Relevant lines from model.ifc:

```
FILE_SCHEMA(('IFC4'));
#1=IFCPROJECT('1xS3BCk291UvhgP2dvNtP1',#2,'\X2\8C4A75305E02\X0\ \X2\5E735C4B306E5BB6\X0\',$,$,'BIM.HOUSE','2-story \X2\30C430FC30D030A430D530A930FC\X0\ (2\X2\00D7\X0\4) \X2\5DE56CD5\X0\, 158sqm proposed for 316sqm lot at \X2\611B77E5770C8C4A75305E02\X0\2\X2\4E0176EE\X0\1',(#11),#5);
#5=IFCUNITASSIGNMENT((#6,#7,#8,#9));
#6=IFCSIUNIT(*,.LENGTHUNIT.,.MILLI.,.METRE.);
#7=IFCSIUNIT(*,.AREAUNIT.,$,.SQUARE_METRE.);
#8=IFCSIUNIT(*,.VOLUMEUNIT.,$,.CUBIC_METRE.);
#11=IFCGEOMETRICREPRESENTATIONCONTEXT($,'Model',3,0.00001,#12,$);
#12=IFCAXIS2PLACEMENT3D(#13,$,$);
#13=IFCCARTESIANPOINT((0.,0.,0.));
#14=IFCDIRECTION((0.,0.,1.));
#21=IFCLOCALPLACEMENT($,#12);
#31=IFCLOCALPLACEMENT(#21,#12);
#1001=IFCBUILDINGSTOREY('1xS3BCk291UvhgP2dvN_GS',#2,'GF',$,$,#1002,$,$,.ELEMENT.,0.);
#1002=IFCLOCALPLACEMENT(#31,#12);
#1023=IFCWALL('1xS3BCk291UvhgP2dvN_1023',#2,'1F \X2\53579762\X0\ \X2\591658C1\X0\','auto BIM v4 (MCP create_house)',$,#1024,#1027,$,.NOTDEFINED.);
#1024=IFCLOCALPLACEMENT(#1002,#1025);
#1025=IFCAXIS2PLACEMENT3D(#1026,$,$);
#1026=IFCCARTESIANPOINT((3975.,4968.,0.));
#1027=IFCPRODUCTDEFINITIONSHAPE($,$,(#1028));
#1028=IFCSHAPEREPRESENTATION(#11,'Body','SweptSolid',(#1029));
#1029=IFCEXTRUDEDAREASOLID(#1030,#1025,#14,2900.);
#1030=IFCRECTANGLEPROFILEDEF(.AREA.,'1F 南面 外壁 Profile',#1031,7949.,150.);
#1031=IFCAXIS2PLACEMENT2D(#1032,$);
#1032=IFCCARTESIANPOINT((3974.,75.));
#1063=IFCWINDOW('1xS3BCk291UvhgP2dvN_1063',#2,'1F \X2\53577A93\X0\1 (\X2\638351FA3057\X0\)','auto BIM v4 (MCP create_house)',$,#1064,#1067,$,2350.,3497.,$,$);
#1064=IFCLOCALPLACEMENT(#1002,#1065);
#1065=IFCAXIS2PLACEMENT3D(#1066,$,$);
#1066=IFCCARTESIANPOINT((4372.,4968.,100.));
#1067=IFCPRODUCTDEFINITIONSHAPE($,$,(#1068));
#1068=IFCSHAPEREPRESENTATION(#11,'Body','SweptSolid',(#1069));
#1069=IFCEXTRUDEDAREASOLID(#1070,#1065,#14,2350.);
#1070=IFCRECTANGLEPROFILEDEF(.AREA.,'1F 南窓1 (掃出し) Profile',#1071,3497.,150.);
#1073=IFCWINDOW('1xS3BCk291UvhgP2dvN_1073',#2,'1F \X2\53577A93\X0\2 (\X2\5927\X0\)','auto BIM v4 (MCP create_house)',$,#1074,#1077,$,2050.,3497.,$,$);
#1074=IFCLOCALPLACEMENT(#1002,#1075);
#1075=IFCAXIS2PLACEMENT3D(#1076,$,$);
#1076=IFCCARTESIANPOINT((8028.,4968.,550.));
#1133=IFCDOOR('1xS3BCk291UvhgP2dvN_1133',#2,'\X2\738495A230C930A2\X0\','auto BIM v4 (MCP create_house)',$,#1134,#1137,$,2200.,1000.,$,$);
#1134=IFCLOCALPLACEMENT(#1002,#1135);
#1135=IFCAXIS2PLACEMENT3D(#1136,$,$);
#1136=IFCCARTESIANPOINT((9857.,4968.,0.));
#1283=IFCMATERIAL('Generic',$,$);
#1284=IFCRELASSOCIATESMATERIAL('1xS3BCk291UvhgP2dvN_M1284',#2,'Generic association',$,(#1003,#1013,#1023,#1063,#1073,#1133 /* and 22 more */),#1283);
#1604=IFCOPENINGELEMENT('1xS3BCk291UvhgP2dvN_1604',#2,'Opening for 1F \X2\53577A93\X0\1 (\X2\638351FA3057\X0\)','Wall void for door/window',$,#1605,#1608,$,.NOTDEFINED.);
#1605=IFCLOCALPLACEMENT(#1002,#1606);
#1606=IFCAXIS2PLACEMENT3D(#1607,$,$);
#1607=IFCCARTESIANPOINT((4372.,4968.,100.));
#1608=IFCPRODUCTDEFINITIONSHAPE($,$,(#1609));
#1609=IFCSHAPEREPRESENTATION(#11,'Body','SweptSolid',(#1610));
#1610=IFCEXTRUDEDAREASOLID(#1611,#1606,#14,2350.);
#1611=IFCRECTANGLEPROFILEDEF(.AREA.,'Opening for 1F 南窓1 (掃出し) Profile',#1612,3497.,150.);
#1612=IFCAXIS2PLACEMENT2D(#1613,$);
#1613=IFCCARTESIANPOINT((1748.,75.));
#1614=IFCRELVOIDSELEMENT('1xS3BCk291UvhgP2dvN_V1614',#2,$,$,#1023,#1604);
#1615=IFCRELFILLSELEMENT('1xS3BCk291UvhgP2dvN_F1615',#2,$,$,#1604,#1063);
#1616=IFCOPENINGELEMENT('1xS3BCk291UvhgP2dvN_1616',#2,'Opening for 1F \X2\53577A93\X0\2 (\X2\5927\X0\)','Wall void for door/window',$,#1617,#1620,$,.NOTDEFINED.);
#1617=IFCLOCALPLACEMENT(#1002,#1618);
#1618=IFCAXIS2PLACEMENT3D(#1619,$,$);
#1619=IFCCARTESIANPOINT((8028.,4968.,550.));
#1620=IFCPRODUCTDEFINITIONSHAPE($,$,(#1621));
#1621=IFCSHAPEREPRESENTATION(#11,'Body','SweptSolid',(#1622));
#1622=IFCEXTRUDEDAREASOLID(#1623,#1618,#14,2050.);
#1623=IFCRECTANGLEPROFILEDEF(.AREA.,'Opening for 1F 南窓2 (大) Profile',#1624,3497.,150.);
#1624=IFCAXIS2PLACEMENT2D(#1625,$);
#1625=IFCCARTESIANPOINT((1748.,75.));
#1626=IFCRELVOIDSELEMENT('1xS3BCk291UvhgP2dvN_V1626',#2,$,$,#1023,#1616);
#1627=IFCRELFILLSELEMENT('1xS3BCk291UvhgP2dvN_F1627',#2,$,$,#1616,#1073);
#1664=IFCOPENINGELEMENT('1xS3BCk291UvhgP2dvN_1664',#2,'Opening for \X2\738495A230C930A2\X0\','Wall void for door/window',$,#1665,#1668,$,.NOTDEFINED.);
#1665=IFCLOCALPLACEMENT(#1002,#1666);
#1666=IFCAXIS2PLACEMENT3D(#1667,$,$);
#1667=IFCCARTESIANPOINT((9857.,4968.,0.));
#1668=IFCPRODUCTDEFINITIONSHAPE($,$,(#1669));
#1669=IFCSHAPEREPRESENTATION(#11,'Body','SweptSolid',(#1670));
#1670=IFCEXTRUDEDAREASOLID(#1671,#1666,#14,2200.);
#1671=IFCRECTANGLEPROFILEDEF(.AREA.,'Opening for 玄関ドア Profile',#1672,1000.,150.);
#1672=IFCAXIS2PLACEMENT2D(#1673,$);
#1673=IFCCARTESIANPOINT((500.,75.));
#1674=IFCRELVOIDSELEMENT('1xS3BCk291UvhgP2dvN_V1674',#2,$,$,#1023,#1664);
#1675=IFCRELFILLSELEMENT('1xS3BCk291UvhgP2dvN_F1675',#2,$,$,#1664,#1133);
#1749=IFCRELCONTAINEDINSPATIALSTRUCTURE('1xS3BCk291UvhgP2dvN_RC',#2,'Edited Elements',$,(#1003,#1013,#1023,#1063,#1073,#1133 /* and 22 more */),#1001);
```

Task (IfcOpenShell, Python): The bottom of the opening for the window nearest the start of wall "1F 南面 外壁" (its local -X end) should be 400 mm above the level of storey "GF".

```python
import numpy as np
import ifcopenshell
import ifcopenshell.api.geometry
import ifcopenshell.geom
import ifcopenshell.util.element
import ifcopenshell.util.placement
import ifcopenshell.util.shape
import ifcopenshell.util.unit

model = ifcopenshell.open("model.ifc")
unit_scale = ifcopenshell.util.unit.calculate_unit_scale(model)

window = model.by_guid("1xS3BCk291UvhgP2dvN_1063")
opening = window.FillsVoids[0].RelatingOpeningElement
storey = ifcopenshell.util.element.get_container(window, ifc_class="IfcBuildingStorey")
level = ifcopenshell.util.placement.get_local_placement(storey.ObjectPlacement)[2, 3]

# The opening's origin need not be at the sill, so measure its lowest point.
shape = ifcopenshell.geom.create_shape(ifcopenshell.geom.settings(), opening)
bottom = ifcopenshell.util.shape.get_shape_bottom_elevation(shape, shape.geometry) / unit_scale
dz = level + 400.0 - bottom

shift = np.array([0.0, 0.0, dz])
# The window is not placed relative to its opening, so move both.
for product in (opening, window):
    matrix = ifcopenshell.util.placement.get_local_placement(product.ObjectPlacement)
    matrix[:3, 3] += shift
    ifcopenshell.api.geometry.edit_object_placement(model, product=product, matrix=matrix, is_si=False)

print(f"moved by {dz * unit_scale:+.3f} m")

model.write("model_v2.ifc")
```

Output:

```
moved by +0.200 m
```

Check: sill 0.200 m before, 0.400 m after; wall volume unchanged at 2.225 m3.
